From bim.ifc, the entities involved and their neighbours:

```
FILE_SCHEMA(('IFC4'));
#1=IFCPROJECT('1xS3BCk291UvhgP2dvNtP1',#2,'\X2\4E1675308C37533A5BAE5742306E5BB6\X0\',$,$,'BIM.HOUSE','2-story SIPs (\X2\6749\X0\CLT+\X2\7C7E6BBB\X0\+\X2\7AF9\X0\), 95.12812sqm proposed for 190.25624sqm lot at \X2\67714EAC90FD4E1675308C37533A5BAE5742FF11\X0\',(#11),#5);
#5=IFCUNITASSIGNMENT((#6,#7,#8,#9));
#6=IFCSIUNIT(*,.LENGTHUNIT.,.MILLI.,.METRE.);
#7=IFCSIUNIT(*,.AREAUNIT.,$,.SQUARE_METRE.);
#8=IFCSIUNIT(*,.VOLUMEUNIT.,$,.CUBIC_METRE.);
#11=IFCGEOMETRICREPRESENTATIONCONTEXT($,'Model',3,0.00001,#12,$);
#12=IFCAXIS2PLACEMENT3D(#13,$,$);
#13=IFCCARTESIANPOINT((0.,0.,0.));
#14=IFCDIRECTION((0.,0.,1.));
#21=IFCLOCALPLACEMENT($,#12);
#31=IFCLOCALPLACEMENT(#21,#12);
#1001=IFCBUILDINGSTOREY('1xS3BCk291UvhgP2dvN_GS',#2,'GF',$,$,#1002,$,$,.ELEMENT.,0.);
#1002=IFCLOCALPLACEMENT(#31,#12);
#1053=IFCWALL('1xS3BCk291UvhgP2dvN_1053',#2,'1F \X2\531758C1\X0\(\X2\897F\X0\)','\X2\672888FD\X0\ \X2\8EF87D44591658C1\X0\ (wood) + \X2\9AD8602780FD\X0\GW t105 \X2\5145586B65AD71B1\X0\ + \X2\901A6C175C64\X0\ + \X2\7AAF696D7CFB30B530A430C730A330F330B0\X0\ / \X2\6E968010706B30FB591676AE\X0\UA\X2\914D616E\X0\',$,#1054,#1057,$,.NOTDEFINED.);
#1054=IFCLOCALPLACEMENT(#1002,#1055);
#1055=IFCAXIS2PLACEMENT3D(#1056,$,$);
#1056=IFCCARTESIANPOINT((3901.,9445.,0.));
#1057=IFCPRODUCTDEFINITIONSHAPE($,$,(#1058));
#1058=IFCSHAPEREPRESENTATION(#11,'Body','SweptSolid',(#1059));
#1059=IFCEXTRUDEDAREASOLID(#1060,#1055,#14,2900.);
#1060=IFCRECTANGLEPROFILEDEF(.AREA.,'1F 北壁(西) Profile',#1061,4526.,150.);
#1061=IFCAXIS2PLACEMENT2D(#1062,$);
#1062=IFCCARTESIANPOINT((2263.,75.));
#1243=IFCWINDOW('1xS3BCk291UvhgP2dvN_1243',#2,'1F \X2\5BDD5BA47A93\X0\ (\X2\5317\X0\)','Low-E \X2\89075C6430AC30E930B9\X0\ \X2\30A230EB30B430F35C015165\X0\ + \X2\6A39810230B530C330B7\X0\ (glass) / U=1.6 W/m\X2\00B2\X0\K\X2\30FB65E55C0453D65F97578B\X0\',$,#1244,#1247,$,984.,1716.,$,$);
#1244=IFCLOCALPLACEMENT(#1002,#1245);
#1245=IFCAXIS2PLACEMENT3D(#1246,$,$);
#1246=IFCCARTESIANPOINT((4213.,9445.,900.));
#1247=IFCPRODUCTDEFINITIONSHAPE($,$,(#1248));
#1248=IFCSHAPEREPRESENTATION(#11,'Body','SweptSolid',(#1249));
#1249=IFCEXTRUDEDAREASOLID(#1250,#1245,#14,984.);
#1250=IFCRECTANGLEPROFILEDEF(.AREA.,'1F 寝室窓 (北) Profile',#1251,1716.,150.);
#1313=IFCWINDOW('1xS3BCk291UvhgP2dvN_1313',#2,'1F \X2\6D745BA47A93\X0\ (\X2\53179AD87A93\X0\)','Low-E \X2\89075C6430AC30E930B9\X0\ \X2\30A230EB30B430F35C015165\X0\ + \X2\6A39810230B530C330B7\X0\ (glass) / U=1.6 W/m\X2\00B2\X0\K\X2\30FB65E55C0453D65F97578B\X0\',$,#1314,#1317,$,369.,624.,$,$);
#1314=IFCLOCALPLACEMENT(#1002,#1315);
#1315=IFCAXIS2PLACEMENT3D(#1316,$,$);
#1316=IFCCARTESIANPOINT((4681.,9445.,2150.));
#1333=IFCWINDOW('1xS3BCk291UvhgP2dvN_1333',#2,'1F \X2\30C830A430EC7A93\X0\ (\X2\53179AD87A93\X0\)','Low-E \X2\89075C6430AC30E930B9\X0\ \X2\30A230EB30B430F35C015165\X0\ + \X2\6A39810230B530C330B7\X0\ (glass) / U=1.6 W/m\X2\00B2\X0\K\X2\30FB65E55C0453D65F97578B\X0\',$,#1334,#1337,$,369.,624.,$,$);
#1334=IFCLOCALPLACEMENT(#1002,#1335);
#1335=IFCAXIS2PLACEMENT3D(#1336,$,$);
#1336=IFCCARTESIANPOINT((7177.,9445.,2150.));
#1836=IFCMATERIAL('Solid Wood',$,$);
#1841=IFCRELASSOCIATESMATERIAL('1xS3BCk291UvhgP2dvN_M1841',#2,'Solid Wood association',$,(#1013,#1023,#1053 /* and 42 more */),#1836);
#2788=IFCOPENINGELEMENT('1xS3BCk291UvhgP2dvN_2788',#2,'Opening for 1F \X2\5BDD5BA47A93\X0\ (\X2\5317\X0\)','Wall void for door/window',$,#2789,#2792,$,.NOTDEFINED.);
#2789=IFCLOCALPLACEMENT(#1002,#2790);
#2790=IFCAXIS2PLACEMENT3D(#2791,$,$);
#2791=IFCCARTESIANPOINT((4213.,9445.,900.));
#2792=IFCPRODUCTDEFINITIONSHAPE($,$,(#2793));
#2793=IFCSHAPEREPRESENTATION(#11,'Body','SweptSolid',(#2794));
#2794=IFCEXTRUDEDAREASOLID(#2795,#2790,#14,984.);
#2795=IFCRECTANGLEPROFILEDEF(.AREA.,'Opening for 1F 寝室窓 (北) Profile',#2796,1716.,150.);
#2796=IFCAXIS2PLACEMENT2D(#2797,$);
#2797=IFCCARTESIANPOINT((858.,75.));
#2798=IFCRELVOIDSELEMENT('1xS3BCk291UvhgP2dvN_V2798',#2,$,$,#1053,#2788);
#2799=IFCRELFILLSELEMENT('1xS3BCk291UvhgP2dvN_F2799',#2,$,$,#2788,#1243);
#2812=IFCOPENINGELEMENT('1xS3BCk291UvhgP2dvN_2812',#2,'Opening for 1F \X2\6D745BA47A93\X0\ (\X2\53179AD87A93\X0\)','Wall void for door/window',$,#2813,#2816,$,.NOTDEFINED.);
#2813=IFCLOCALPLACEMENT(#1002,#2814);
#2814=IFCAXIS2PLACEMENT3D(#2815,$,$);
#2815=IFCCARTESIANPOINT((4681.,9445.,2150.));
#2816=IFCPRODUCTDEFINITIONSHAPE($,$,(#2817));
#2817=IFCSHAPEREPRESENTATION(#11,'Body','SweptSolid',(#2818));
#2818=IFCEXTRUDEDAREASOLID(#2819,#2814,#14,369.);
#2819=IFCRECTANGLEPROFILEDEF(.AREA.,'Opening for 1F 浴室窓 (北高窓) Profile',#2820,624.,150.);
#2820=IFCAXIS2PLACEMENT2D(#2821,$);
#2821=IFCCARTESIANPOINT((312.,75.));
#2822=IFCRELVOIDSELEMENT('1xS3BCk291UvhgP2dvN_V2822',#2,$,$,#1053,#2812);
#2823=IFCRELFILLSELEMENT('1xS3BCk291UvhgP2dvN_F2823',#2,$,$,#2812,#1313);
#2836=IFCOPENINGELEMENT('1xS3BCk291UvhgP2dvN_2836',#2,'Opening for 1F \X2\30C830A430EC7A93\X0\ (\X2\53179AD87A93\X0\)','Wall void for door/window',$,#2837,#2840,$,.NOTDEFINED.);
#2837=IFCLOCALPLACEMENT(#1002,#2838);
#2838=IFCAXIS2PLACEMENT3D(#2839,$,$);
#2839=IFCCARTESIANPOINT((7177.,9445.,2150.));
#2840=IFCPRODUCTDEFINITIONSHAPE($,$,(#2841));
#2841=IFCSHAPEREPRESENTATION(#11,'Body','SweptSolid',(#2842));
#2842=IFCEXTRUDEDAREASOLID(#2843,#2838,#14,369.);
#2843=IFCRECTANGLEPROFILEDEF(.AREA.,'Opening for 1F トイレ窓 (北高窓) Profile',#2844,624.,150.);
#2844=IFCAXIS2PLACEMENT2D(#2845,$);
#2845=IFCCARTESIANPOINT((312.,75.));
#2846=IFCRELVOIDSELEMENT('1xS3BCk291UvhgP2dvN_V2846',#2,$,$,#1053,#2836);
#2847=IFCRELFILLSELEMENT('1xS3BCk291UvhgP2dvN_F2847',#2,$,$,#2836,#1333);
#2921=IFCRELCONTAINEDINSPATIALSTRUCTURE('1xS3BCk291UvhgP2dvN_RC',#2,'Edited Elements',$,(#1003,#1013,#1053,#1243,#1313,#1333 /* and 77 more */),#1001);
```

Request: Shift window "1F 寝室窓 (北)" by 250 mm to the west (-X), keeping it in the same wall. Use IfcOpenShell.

```python
import ifcopenshell
import ifcopenshell.api.geometry
import ifcopenshell.util.placement
import ifcopenshell.util.unit

model = ifcopenshell.open("bim.ifc")
unit_scale = ifcopenshell.util.unit.calculate_unit_scale(model)

window = model.by_guid("1xS3BCk291UvhgP2dvN_1243")
opening = window.FillsVoids[0].RelatingOpeningElement
wall = opening.VoidsElements[0].RelatingBuildingElement

wall_matrix = ifcopenshell.util.placement.get_local_placement(wall.ObjectPlacement)
shift = wall_matrix[:3, 0] * -0.25 / unit_scale
before = ifcopenshell.util.placement.get_local_placement(window.ObjectPlacement)[:3, 3].copy()

# The window is not placed relative to its opening, so move both.
for product in (opening, window):
    matrix = ifcopenshell.util.placement.get_local_placement(product.ObjectPlacement)
    matrix[:3, 3] += shift
    ifcopenshell.api.geometry.edit_object_placement(model, product=product, matrix=matrix, is_si=False)

after = ifcopenshell.util.placement.get_local_placement(window.ObjectPlacement)[:3, 3]
print("window moved by", (after - before).round(3) + 0.0)

model.write("bim_edited.ifc")
```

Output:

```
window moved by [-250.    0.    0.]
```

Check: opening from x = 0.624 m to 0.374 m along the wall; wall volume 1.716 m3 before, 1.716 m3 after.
